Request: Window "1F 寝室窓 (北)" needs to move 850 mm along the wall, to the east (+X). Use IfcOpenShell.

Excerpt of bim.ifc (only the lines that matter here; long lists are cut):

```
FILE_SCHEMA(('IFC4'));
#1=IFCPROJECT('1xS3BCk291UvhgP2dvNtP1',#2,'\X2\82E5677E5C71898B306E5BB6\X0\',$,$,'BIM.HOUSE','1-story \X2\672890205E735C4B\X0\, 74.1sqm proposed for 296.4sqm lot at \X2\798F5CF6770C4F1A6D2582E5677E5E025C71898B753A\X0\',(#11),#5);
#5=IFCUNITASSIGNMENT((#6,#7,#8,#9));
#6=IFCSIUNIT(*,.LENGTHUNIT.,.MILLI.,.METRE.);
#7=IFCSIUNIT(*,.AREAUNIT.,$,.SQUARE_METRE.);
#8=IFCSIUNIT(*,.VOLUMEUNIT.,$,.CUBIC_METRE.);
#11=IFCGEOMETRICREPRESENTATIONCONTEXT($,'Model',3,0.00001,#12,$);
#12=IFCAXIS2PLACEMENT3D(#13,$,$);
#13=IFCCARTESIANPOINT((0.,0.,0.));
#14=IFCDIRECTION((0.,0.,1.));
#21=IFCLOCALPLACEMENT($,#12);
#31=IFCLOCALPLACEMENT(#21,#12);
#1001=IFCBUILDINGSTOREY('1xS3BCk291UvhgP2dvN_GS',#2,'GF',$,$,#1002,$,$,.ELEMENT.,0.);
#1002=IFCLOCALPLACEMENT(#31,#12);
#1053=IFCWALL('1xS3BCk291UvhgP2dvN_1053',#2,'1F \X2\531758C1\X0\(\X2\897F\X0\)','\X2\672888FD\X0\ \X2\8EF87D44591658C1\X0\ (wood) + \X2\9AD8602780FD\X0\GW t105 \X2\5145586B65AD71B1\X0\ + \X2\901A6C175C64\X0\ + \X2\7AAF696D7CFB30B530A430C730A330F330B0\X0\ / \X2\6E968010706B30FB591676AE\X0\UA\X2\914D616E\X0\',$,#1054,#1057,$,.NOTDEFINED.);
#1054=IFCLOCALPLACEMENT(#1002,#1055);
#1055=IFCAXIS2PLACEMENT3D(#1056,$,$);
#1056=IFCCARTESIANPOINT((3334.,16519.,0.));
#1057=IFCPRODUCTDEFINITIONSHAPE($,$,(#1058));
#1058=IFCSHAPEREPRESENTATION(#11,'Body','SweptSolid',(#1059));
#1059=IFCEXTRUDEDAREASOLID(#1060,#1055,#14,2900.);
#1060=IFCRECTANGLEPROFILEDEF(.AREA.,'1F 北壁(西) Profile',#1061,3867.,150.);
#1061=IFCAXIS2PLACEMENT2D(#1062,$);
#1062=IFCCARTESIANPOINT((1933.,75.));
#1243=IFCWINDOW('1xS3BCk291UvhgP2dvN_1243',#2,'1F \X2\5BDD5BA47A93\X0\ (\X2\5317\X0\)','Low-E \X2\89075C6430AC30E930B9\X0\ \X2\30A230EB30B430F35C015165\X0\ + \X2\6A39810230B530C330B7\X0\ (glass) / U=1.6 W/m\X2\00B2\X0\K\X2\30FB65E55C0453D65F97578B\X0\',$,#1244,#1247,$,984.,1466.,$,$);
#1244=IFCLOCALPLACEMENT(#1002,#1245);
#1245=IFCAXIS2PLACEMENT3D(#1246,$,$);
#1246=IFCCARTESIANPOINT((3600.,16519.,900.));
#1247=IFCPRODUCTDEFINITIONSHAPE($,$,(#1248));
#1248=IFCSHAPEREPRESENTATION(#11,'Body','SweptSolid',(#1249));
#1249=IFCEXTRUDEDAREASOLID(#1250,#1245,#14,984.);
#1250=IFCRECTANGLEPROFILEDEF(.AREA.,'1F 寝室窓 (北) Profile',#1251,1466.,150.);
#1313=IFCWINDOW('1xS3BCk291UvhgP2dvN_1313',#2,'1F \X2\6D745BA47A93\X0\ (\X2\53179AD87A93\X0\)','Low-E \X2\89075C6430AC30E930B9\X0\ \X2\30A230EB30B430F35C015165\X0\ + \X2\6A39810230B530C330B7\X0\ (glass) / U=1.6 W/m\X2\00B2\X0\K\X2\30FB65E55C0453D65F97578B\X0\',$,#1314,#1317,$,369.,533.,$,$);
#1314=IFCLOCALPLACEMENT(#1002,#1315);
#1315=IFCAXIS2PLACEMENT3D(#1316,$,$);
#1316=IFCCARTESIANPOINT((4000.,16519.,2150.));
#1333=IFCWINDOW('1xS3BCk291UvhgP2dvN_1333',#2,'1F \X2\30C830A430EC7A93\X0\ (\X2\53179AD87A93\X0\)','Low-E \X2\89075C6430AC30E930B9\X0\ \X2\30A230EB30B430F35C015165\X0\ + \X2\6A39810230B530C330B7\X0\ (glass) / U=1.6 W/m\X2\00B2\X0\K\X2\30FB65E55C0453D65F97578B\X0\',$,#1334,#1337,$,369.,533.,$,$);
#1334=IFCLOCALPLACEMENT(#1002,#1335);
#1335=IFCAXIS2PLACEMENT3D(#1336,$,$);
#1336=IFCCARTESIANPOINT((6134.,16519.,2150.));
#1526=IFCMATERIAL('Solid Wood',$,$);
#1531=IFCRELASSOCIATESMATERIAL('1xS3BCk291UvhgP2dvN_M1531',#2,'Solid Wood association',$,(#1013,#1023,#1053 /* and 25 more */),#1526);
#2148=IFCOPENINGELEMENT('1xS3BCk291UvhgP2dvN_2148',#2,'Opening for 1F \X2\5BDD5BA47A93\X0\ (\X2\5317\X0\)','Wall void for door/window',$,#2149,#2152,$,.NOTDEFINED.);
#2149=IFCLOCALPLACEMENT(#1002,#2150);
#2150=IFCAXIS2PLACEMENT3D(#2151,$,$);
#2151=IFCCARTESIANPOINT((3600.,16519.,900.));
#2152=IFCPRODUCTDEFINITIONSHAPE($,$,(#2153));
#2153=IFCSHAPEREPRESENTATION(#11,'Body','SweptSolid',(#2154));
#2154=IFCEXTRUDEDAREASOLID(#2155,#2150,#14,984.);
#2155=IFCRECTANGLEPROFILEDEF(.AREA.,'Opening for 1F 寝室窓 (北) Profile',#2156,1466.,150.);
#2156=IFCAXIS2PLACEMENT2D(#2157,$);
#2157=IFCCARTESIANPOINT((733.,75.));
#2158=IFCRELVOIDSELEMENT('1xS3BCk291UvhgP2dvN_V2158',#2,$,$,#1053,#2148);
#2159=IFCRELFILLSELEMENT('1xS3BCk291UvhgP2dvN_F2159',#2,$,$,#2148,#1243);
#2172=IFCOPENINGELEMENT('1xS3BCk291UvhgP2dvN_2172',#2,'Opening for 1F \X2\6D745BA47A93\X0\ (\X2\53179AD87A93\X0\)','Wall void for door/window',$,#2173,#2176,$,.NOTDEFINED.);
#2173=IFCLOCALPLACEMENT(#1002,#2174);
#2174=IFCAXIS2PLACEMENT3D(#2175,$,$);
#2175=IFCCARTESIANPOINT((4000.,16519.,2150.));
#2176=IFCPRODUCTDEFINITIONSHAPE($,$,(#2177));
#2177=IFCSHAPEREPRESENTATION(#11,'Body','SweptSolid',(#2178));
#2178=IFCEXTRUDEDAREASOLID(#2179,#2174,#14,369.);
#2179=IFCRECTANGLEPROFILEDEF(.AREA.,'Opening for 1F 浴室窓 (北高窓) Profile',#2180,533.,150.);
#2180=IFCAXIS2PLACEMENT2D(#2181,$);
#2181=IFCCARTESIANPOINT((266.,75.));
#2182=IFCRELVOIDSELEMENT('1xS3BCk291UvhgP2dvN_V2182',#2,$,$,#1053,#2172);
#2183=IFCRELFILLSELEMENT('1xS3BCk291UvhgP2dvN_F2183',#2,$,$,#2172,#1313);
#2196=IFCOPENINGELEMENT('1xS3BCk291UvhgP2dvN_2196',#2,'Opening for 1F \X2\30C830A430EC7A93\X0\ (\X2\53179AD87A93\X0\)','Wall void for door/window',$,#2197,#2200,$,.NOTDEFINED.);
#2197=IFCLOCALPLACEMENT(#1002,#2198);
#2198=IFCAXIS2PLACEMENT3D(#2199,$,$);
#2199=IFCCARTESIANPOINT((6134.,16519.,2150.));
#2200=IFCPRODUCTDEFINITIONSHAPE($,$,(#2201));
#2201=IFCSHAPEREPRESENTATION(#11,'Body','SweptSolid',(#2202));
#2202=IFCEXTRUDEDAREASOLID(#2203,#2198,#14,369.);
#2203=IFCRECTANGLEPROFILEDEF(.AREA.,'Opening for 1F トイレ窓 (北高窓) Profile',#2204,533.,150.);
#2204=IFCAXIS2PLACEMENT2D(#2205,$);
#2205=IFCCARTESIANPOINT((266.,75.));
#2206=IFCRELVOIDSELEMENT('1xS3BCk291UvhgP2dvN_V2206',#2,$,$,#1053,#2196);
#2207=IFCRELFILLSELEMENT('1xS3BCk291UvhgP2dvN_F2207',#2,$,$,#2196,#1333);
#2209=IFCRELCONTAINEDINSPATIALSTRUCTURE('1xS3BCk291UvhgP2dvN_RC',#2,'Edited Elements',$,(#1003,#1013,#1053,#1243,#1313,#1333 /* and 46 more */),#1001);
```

```python
import ifcopenshell
import ifcopenshell.api.geometry
import ifcopenshell.util.placement

model = ifcopenshell.open("bim.ifc")

window = model.by_id(1243)
opening = window.FillsVoids[0].RelatingOpeningElement
wall = opening.VoidsElements[0].RelatingBuildingElement

wall_matrix = ifcopenshell.util.placement.get_local_placement(wall.ObjectPlacement)
shift = wall_matrix[:3, 0] * 850.0
before = ifcopenshell.util.placement.get_local_placement(window.ObjectPlacement)[:3, 3].copy()

# The window is not placed relative to its opening, so move both.
for product in (opening, window):
    matrix = ifcopenshell.util.placement.get_local_placement(product.ObjectPlacement)
    matrix[:3, 3] += shift
    ifcopenshell.api.geometry.edit_object_placement(model, product=product, matrix=matrix, is_si=False)

after = ifcopenshell.util.placement.get_local_placement(window.ObjectPlacement)[:3, 3]
print("window moved by", (after - before).round(3) + 0.0)

model.write("bim-out.ifc")
```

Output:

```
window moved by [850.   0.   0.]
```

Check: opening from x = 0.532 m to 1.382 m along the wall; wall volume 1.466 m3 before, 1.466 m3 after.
